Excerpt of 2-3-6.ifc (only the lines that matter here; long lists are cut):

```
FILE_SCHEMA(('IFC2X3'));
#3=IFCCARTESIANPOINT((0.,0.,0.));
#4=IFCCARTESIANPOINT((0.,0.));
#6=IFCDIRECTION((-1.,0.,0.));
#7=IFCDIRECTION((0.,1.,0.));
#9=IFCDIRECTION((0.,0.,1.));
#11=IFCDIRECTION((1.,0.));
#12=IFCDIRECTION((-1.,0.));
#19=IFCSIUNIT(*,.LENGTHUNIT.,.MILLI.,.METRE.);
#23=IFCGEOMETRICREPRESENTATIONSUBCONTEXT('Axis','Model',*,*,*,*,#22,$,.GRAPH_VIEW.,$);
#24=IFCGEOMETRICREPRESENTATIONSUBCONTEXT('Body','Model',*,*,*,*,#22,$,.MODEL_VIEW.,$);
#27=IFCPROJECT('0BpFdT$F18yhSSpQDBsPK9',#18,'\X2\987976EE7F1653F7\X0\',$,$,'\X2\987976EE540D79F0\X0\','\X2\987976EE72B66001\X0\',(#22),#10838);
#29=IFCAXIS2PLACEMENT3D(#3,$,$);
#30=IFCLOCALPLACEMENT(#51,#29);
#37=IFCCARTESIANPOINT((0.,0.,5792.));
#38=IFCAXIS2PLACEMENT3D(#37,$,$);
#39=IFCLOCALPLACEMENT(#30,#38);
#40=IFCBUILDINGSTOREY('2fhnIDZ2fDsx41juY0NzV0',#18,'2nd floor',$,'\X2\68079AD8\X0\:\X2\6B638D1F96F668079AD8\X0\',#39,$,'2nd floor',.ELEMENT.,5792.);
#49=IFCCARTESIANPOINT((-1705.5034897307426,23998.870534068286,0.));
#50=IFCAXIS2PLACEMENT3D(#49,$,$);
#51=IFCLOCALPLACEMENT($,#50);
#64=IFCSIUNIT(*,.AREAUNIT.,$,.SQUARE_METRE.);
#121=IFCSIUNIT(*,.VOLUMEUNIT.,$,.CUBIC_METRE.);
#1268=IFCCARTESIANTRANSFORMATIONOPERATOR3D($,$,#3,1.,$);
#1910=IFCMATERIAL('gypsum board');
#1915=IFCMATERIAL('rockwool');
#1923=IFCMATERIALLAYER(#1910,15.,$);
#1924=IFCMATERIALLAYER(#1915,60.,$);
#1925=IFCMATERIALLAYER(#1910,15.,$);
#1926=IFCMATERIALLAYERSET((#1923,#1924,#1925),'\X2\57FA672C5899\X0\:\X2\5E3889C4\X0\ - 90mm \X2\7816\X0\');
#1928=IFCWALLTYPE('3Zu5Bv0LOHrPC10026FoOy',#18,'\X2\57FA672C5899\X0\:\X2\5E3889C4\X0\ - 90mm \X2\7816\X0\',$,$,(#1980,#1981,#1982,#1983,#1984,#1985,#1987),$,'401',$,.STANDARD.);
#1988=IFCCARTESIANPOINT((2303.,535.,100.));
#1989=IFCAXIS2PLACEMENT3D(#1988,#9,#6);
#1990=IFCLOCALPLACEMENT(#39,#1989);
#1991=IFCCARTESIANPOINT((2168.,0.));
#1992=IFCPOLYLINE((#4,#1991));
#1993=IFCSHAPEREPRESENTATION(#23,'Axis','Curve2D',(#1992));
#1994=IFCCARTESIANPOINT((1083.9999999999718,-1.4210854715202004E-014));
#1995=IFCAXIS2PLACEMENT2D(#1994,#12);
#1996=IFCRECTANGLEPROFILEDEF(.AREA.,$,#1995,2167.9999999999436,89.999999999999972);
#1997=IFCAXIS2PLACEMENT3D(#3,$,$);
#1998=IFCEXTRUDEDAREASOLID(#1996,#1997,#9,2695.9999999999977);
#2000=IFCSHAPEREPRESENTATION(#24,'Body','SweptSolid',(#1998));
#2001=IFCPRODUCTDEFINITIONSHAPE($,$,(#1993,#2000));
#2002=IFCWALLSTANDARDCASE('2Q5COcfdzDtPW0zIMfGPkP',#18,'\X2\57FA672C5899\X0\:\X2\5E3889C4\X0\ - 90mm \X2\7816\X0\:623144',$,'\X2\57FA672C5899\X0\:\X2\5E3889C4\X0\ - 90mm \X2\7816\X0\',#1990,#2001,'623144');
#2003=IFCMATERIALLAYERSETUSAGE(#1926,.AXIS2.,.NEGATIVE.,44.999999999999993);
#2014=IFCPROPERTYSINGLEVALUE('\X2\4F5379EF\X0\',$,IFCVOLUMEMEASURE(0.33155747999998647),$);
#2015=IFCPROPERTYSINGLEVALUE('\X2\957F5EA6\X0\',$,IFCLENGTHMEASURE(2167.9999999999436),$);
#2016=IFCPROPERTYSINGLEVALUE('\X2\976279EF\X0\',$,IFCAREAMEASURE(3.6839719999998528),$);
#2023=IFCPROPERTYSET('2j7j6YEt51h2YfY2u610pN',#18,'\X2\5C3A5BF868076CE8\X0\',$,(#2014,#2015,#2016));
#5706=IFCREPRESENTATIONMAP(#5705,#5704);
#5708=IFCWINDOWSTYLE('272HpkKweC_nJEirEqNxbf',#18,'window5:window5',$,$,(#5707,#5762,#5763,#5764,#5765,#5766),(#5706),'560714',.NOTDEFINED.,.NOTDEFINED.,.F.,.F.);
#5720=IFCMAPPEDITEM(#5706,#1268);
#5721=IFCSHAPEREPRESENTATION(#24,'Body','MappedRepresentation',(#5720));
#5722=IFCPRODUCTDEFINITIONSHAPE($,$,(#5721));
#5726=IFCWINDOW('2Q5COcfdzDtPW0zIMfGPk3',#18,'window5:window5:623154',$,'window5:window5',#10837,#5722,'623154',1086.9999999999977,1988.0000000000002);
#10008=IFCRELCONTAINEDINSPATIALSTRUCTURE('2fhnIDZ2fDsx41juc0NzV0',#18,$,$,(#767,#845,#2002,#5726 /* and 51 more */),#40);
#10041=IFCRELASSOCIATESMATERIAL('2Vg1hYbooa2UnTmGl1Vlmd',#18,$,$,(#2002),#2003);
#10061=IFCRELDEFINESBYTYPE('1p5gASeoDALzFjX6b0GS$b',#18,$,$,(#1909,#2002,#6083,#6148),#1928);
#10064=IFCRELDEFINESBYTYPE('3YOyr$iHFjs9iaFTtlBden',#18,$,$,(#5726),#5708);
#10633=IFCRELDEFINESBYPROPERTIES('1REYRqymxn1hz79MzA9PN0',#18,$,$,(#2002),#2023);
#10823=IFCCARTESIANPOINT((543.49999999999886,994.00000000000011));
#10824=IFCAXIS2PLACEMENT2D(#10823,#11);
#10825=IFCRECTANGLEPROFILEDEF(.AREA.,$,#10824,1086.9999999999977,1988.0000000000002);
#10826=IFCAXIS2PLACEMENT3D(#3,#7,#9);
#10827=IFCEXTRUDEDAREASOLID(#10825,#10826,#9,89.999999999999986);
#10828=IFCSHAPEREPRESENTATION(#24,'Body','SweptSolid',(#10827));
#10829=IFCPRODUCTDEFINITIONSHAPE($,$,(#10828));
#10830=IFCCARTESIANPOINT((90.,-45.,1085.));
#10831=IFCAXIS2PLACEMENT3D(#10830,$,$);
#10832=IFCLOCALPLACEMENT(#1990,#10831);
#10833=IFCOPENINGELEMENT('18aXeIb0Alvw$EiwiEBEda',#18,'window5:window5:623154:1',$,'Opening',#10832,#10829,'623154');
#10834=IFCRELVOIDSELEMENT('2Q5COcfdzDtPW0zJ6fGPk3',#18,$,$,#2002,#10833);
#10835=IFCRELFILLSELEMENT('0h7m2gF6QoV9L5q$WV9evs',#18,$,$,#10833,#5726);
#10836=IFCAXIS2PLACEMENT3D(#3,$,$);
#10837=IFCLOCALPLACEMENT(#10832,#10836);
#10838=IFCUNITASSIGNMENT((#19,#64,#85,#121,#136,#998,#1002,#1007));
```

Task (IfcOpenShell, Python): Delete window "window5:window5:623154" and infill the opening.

```python
import ifcopenshell
import ifcopenshell.api.feature
import ifcopenshell.api.pset
import ifcopenshell.api.root
import ifcopenshell.geom
import ifcopenshell.util.element
import ifcopenshell.util.shape
import ifcopenshell.util.unit

model = ifcopenshell.open("2-3-6.ifc")
area_scale = ifcopenshell.util.unit.calculate_unit_scale(model, "AREAUNIT")
volume_scale = ifcopenshell.util.unit.calculate_unit_scale(model, "VOLUMEUNIT")
settings = ifcopenshell.geom.settings()


def volume(element):
    """Net volume in cubic metres, openings subtracted."""
    shape = ifcopenshell.geom.create_shape(settings, element)
    return ifcopenshell.util.shape.get_volume(shape.geometry)


window = model.by_guid("2Q5COcfdzDtPW0zIMfGPk3")
opening = window.FillsVoids[0].RelatingOpeningElement
wall = opening.VoidsElements[0].RelatingBuildingElement
before = volume(wall)

ifcopenshell.api.root.remove_product(model, product=window)
ifcopenshell.api.feature.remove_feature(model, feature=opening)

after = volume(wall)
thickness = 0.09  # wall thickness in metres

# Update the wall's stored quantities.
pset = model.by_id(ifcopenshell.util.element.get_pset(wall, "尺寸标注", should_inherit=False)["id"])
ifcopenshell.api.pset.edit_pset(model, pset=pset, properties={
    "体积": model.create_entity("IfcVolumeMeasure", after / volume_scale),
    "面积": model.create_entity("IfcAreaMeasure", after / thickness / area_scale),
})

print(f"wall volume {before:.3f} -> {after:.3f} m3")

model.write("2-3-6_edited.ifc")
```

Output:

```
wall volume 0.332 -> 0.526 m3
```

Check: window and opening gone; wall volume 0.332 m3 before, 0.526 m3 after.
